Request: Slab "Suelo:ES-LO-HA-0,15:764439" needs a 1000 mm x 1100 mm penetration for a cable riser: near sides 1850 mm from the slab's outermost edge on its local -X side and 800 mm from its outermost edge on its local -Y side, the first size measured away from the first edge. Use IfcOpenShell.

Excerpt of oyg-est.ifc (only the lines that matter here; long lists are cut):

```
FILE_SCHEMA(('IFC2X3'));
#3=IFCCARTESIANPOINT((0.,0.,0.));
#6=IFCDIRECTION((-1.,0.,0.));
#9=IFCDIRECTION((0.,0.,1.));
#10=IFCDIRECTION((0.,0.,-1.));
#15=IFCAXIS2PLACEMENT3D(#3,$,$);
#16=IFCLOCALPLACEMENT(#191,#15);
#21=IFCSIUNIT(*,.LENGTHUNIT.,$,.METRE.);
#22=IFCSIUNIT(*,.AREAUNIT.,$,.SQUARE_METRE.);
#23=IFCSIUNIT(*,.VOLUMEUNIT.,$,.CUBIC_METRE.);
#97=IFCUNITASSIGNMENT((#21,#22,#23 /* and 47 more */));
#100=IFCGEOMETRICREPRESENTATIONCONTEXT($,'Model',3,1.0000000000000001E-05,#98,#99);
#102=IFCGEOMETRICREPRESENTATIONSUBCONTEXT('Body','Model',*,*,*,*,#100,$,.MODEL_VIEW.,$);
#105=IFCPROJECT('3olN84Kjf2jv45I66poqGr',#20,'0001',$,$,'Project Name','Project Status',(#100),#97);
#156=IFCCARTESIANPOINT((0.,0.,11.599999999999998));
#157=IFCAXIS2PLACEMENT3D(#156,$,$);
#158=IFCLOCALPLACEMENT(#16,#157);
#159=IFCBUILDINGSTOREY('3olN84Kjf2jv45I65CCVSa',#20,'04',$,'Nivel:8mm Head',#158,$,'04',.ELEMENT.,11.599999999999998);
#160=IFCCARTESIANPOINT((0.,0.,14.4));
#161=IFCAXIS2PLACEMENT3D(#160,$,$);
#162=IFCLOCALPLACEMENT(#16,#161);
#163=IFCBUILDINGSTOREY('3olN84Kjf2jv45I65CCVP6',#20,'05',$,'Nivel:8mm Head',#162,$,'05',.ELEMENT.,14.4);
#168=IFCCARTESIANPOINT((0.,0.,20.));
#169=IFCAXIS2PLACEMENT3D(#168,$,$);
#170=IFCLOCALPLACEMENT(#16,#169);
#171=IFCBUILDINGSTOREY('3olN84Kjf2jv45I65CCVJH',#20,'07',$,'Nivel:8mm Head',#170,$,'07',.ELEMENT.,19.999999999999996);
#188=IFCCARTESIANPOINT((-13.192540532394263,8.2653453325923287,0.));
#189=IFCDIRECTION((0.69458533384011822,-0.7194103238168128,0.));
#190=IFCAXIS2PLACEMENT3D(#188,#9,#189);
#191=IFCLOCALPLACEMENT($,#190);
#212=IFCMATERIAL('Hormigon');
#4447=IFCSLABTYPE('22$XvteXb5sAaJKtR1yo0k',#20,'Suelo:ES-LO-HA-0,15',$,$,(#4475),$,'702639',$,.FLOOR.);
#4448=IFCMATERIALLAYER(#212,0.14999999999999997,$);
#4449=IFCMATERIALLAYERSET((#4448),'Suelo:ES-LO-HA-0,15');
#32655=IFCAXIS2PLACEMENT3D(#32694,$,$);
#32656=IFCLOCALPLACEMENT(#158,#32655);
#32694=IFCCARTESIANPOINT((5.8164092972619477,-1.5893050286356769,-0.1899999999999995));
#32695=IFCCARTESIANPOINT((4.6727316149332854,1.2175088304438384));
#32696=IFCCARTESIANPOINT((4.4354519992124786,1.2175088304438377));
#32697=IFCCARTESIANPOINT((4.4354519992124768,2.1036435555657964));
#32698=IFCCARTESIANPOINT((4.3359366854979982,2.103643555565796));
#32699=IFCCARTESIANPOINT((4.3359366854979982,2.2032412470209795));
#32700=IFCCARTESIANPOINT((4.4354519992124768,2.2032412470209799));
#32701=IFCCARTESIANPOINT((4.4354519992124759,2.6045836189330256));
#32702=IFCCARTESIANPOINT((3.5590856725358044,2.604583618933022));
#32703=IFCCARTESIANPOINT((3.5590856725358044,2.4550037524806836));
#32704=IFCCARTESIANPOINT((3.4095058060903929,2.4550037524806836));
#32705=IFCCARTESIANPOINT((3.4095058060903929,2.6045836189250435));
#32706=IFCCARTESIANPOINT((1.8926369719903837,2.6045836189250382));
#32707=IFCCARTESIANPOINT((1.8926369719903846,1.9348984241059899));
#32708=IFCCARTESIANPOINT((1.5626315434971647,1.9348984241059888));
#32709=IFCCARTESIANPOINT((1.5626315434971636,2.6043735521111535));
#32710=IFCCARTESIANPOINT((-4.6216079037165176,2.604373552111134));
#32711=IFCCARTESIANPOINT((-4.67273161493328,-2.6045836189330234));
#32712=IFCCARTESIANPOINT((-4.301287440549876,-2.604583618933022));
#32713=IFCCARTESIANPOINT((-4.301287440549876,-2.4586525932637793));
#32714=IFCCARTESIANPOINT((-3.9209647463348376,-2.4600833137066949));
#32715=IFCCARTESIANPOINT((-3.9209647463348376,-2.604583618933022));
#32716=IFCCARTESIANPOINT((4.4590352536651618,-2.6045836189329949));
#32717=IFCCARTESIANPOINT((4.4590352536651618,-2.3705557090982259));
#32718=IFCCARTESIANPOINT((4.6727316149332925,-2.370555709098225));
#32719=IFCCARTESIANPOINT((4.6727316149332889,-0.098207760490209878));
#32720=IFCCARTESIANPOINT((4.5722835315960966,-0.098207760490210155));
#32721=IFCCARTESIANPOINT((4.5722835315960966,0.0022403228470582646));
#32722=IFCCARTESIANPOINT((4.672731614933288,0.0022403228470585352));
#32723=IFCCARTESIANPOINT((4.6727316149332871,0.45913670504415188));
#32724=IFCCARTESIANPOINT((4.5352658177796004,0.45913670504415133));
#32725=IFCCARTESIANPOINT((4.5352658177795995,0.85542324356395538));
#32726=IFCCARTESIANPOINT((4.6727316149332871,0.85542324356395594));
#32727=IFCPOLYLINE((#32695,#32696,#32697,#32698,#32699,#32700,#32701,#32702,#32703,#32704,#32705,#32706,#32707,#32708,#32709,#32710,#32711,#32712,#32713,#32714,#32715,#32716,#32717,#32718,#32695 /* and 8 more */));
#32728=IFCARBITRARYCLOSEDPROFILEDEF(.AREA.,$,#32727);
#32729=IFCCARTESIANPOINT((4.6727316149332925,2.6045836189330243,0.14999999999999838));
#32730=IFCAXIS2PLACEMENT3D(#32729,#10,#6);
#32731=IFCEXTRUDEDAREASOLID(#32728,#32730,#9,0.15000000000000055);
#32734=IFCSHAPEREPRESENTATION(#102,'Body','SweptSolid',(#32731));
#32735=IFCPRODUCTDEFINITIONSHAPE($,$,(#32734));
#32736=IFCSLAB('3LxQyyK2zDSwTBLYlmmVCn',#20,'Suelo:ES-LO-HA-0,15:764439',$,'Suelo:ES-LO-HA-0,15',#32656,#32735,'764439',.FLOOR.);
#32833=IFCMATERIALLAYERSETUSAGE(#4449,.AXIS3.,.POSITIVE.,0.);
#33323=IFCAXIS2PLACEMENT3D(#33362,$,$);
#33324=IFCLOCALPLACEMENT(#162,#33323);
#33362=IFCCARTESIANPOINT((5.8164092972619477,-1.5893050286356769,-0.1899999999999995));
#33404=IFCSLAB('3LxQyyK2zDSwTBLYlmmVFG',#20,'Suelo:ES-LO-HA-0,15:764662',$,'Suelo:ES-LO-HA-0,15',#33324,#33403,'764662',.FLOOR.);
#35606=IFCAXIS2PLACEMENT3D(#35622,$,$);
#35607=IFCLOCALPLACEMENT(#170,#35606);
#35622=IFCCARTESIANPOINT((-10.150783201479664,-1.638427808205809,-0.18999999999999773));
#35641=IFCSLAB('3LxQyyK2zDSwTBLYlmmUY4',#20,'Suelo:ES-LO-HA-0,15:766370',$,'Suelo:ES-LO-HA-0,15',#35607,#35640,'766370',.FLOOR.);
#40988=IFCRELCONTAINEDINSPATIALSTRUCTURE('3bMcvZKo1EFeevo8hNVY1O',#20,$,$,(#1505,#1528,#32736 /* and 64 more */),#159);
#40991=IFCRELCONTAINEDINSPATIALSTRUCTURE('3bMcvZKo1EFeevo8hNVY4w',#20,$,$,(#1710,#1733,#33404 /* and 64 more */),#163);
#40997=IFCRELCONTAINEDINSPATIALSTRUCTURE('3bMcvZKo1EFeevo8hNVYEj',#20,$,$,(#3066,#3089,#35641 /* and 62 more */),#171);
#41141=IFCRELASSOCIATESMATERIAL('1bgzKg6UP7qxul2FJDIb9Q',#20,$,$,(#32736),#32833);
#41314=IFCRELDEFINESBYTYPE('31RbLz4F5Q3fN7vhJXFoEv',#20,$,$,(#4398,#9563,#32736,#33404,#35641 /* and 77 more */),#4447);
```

```python
import numpy as np
import ifcopenshell
import ifcopenshell.api.feature
import ifcopenshell.api.geometry
import ifcopenshell.api.root
import ifcopenshell.geom
import ifcopenshell.util.placement
import ifcopenshell.util.representation
import ifcopenshell.util.shape
import ifcopenshell.util.unit

model = ifcopenshell.open("oyg-est.ifc")
unit_scale = ifcopenshell.util.unit.calculate_unit_scale(model)
settings = ifcopenshell.geom.settings()


def volume(element):
    """Net volume in cubic metres, openings subtracted."""
    shape = ifcopenshell.geom.create_shape(settings, element)
    return ifcopenshell.util.shape.get_volume(shape.geometry)


slab = model.by_guid("3LxQyyK2zDSwTBLYlmmVCn")
before = volume(slab)

# Extent in the slab's own axes, in metres. The edges named are its -X and -Y sides.
slab_shape = ifcopenshell.geom.create_shape(settings, slab)
vertices = ifcopenshell.util.shape.get_vertices(slab_shape.geometry)
x_min, y_min, bottom = vertices.min(axis=0)
top = vertices[:, 2].max()

opening = ifcopenshell.api.root.create_entity(model, ifc_class="IfcOpeningElement", name="Cable riser opening")
context = ifcopenshell.util.representation.get_context(model, "Model", "Body", "MODEL_VIEW")
width, depth = 1, 1.1
outline = [(0.0, 0.0), (width, 0.0), (width, depth), (0.0, depth), (0.0, 0.0)]
# Overshoot both faces by 50 mm so the cut is clean.
shape = ifcopenshell.api.geometry.add_slab_representation(
    model, context=context, depth=top - bottom + 0.1, polyline=outline
)
ifcopenshell.api.geometry.assign_representation(model, product=opening, representation=shape)

matrix = ifcopenshell.util.placement.get_local_placement(slab.ObjectPlacement)
matrix[:, 3] = matrix @ np.append(np.array([x_min + 1.85, y_min + 0.8, bottom - 0.05]) / unit_scale, 1.0)
ifcopenshell.api.geometry.edit_object_placement(model, product=opening, matrix=matrix, is_si=False)
ifcopenshell.api.feature.add_feature(model, feature=opening, element=slab)

after = volume(slab)

print(f"slab volume {before:.3f} -> {after:.3f} m3")

model.write("oyg-est_v2.ifc")
```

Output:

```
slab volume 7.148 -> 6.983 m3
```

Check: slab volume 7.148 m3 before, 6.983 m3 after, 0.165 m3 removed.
